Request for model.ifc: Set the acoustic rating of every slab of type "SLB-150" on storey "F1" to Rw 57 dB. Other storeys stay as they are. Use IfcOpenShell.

First a look at what the model holds.

```python
import ifcopenshell
import ifcopenshell.util.element

model = ifcopenshell.open("model.ifc")
print(model.schema)
storey = next(s for s in model.by_type("IfcBuildingStorey") if s.Name == "F1")
slabs = [e for e in ifcopenshell.util.element.get_decomposition(storey) if e.is_a("IfcSlab")]
seen = {}
for e in slabs:
    element_type = ifcopenshell.util.element.get_type(e)
    key = (element_type.Name if element_type != e and element_type else None, ifcopenshell.util.element.get_pset(e, "Pset_SlabCommon", "AcousticRating"))
    seen[key] = seen.get(key, 0) + 1
for (name, value), count in sorted(seen.items(), key=str):
    print(count, "x", name, "|", value)
```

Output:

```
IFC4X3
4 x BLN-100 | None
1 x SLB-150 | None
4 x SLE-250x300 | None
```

```python
import ifcopenshell
import ifcopenshell.api.pset
import ifcopenshell.util.element

model = ifcopenshell.open("model.ifc")

storey = next(s for s in model.by_type("IfcBuildingStorey") if s.Name == "F1")
slabs = [e for e in ifcopenshell.util.element.get_decomposition(storey) if e.is_a("IfcSlab")]

count = 0
for e in slabs:
    element_type = ifcopenshell.util.element.get_type(e)
    if element_type in (None, e) or element_type.Name != "SLB-150":
        continue
    # add_pset returns the element's existing set when there is one.
    pset = ifcopenshell.api.pset.add_pset(model, product=e, name="Pset_SlabCommon")
    ifcopenshell.api.pset.edit_pset(model, pset=pset, properties={"AcousticRating": "Rw 57 dB"})
    count += 1

print(count, "slabs updated")

model.write("model-out.ifc")
```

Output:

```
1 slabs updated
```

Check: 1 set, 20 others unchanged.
